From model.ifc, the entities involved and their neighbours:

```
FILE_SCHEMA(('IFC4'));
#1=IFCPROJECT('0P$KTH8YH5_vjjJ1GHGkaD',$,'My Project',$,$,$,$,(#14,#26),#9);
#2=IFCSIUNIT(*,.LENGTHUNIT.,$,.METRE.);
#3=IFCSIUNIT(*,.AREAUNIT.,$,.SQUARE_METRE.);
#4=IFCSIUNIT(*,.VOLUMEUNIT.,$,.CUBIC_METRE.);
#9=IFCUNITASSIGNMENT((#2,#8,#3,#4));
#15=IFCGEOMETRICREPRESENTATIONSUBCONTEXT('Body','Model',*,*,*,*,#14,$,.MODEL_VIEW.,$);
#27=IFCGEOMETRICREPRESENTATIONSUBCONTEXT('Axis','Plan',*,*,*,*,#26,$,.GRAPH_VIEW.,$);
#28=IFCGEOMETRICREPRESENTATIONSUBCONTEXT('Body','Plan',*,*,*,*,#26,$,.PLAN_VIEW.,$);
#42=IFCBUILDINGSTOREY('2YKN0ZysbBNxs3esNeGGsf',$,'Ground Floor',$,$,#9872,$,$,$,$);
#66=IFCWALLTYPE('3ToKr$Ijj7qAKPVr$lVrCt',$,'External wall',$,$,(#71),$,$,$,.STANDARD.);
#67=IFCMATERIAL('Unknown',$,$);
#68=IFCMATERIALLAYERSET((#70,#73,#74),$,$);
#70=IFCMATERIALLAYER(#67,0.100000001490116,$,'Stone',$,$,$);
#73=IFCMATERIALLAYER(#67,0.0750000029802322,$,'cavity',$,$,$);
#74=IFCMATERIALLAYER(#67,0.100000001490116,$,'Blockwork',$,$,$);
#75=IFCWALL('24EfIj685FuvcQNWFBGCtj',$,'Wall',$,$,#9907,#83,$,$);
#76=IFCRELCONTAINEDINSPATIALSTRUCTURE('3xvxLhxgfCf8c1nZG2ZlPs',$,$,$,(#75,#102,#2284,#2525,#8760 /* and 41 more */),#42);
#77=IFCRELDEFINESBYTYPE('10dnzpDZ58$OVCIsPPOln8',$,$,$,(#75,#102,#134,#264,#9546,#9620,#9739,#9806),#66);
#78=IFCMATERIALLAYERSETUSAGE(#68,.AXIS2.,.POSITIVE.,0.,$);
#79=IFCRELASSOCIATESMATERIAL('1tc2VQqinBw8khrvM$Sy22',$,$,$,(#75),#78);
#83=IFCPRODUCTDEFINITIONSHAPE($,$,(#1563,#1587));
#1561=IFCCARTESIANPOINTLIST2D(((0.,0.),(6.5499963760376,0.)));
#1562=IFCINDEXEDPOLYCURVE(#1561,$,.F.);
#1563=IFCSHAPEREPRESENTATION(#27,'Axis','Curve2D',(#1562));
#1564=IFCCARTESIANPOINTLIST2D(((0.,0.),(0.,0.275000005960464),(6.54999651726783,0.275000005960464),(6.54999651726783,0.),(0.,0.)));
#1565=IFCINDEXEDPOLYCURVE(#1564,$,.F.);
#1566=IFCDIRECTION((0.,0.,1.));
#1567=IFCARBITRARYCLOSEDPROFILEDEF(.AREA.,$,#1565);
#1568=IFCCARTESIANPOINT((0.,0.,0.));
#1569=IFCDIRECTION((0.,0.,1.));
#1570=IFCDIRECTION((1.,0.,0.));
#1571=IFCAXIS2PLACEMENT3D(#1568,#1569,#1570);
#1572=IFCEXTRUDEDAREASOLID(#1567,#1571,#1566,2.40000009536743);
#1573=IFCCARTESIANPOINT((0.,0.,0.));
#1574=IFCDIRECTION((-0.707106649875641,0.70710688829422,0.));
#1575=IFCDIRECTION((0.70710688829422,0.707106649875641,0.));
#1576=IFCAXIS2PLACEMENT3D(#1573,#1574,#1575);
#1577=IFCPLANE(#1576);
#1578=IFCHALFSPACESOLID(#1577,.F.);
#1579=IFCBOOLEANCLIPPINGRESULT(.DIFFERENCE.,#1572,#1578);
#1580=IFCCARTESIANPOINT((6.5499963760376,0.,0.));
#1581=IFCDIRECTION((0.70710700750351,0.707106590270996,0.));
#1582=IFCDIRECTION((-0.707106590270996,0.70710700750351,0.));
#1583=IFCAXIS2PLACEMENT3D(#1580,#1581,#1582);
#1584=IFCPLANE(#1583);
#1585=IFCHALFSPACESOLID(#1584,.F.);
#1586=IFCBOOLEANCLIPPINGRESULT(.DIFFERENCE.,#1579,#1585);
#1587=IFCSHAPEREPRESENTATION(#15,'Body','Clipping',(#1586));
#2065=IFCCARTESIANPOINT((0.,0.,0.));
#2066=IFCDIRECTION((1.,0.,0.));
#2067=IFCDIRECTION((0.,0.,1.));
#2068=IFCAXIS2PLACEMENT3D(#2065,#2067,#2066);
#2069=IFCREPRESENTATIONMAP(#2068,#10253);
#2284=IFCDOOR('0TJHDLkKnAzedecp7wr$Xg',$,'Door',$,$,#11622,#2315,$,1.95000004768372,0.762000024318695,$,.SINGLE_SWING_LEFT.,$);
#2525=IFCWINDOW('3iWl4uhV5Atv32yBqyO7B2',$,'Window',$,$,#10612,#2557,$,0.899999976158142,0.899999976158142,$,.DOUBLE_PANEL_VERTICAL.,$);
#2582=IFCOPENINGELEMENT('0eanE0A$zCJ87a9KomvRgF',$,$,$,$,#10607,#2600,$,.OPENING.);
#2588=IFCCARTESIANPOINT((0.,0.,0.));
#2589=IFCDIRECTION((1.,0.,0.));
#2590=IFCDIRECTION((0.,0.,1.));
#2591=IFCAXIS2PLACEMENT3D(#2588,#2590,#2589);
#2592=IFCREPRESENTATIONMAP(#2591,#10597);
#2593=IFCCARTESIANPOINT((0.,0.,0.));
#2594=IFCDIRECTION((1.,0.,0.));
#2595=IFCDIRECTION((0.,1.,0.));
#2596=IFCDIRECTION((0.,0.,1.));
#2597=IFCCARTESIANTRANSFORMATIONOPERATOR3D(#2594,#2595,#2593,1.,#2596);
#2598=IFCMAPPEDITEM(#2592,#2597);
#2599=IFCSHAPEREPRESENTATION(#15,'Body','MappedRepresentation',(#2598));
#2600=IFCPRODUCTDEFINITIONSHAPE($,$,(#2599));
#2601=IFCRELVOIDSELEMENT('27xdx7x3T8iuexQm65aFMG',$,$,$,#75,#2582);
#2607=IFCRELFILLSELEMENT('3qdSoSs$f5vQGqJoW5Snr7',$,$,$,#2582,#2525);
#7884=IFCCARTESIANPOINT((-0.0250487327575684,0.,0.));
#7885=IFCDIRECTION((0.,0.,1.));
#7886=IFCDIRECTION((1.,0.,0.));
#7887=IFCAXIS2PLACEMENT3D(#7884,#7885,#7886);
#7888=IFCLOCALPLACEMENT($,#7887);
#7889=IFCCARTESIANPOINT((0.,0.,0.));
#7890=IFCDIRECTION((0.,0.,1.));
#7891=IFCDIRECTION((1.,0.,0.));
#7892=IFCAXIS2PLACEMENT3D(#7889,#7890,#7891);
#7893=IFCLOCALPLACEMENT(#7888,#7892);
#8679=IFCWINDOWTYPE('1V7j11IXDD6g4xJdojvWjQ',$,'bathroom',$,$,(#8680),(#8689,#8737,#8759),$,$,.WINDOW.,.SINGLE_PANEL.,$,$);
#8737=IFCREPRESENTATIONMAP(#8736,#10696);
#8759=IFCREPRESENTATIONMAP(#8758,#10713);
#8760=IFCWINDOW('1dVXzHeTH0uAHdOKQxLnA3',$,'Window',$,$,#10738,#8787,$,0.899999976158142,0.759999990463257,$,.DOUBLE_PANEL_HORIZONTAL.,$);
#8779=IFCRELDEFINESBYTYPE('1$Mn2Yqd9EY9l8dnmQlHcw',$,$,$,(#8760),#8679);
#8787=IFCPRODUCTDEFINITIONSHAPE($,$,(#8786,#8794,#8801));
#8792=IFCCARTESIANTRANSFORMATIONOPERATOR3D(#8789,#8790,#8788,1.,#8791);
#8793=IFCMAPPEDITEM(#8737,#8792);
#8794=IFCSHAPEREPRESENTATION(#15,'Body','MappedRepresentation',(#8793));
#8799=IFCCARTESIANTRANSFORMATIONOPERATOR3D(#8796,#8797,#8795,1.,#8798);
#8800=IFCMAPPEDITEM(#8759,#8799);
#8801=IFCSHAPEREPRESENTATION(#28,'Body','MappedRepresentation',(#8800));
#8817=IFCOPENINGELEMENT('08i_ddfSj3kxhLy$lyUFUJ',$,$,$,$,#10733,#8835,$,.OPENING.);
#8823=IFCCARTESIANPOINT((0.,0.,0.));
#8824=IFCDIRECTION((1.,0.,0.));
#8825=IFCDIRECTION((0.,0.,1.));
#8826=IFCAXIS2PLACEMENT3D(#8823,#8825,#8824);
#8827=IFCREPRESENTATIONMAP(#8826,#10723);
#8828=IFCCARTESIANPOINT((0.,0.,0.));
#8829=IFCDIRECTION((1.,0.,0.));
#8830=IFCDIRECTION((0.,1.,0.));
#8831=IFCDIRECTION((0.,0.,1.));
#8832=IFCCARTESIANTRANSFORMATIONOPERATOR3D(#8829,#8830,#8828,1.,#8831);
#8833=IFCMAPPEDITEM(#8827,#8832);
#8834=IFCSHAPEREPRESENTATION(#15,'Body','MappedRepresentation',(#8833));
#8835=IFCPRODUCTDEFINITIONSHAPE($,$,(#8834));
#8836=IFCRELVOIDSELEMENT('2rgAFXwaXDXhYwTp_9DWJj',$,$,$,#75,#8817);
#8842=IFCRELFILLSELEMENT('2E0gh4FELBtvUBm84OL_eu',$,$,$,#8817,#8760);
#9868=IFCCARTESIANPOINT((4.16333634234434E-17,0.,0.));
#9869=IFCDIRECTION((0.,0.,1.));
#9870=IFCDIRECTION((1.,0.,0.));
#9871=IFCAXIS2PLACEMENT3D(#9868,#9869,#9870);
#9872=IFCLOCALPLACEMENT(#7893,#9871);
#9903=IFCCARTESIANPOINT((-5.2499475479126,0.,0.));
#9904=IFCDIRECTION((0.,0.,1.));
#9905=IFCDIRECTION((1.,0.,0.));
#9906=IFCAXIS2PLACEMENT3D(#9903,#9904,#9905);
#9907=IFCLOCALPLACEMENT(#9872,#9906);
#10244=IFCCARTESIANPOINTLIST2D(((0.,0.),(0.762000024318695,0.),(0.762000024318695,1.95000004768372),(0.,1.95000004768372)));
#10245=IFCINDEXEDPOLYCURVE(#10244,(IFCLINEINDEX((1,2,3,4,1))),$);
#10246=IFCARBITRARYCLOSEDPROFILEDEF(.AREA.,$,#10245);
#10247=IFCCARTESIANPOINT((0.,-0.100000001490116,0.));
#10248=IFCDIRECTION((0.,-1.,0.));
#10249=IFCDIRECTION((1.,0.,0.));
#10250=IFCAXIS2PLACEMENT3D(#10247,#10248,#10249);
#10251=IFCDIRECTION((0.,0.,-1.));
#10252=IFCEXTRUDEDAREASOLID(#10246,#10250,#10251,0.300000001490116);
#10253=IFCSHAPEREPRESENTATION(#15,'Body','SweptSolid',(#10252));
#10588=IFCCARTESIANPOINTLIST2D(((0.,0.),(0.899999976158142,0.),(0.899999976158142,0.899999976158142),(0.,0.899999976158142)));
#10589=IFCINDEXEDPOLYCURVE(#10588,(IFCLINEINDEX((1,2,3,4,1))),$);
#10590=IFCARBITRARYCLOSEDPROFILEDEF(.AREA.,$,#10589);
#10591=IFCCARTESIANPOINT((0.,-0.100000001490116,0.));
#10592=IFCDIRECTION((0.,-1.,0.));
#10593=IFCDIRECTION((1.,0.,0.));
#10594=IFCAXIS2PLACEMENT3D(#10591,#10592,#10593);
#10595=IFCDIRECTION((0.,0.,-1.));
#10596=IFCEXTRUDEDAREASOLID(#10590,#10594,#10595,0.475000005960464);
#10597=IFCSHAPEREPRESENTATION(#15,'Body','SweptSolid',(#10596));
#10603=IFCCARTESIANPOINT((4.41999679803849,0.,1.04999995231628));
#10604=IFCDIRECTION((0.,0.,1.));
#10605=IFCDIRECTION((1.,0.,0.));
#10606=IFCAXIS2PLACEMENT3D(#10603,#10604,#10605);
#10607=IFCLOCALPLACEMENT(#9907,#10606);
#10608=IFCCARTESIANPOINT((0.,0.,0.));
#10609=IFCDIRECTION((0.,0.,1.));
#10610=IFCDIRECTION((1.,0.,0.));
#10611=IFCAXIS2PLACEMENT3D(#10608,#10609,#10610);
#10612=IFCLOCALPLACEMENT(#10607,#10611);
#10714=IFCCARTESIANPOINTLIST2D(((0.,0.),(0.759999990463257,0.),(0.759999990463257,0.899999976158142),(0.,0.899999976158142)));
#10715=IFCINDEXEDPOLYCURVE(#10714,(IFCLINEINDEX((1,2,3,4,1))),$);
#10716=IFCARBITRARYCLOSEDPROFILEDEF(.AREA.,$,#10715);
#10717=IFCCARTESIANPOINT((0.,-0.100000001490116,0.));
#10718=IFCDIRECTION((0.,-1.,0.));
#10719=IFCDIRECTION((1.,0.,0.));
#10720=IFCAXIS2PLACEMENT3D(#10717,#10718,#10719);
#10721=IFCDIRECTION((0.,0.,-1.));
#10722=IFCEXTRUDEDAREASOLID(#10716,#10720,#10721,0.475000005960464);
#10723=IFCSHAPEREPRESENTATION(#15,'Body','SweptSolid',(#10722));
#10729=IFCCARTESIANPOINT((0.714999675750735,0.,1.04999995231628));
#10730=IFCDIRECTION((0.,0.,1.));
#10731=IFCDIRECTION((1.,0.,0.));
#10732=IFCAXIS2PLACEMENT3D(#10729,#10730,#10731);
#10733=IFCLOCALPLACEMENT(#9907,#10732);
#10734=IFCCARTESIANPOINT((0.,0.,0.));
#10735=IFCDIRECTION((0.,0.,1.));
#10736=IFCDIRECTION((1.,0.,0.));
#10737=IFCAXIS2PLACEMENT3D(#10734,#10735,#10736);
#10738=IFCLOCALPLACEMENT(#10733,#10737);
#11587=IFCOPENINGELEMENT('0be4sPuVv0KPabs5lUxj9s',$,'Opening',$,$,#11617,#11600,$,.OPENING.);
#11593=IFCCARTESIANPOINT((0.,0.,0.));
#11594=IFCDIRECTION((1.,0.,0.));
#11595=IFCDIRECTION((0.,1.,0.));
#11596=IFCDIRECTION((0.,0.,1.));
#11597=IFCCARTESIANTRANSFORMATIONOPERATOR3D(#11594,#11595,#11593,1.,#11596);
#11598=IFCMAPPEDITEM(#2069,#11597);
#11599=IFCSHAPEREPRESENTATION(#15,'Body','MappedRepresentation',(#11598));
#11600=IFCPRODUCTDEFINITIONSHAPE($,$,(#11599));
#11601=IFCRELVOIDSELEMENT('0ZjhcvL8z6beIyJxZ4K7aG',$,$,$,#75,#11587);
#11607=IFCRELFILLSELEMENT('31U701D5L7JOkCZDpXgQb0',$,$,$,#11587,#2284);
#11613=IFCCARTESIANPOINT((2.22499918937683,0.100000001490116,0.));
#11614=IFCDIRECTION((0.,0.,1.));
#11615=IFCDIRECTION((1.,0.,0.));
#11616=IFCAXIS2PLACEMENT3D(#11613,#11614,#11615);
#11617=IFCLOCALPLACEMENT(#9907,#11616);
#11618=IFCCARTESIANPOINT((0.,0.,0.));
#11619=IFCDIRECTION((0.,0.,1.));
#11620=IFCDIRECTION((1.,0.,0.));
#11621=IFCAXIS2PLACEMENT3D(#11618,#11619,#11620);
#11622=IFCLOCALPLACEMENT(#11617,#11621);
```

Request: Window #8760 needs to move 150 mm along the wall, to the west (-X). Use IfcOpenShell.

```python
import ifcopenshell
import ifcopenshell.api.geometry
import ifcopenshell.util.placement
import ifcopenshell.util.unit

model = ifcopenshell.open("model.ifc")
unit_scale = ifcopenshell.util.unit.calculate_unit_scale(model)

window = model.by_guid("1dVXzHeTH0uAHdOKQxLnA3")
opening = window.FillsVoids[0].RelatingOpeningElement
wall = opening.VoidsElements[0].RelatingBuildingElement

wall_matrix = ifcopenshell.util.placement.get_local_placement(wall.ObjectPlacement)
shift = wall_matrix[:3, 0] * -0.15 / unit_scale
before = ifcopenshell.util.placement.get_local_placement(window.ObjectPlacement)[:3, 3].copy()

# The window is placed relative to its opening, so it follows when the opening moves.
matrix = ifcopenshell.util.placement.get_local_placement(opening.ObjectPlacement)
matrix[:3, 3] += shift
ifcopenshell.api.geometry.edit_object_placement(
    model, product=opening, matrix=matrix, is_si=False, should_transform_children=True
)

after = ifcopenshell.util.placement.get_local_placement(window.ObjectPlacement)[:3, 3]
print("window moved by", (after - before).round(3) + 0.0)

model.write("model_v2.ifc")
```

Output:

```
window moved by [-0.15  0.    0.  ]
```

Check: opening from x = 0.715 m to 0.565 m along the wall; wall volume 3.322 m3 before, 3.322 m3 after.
